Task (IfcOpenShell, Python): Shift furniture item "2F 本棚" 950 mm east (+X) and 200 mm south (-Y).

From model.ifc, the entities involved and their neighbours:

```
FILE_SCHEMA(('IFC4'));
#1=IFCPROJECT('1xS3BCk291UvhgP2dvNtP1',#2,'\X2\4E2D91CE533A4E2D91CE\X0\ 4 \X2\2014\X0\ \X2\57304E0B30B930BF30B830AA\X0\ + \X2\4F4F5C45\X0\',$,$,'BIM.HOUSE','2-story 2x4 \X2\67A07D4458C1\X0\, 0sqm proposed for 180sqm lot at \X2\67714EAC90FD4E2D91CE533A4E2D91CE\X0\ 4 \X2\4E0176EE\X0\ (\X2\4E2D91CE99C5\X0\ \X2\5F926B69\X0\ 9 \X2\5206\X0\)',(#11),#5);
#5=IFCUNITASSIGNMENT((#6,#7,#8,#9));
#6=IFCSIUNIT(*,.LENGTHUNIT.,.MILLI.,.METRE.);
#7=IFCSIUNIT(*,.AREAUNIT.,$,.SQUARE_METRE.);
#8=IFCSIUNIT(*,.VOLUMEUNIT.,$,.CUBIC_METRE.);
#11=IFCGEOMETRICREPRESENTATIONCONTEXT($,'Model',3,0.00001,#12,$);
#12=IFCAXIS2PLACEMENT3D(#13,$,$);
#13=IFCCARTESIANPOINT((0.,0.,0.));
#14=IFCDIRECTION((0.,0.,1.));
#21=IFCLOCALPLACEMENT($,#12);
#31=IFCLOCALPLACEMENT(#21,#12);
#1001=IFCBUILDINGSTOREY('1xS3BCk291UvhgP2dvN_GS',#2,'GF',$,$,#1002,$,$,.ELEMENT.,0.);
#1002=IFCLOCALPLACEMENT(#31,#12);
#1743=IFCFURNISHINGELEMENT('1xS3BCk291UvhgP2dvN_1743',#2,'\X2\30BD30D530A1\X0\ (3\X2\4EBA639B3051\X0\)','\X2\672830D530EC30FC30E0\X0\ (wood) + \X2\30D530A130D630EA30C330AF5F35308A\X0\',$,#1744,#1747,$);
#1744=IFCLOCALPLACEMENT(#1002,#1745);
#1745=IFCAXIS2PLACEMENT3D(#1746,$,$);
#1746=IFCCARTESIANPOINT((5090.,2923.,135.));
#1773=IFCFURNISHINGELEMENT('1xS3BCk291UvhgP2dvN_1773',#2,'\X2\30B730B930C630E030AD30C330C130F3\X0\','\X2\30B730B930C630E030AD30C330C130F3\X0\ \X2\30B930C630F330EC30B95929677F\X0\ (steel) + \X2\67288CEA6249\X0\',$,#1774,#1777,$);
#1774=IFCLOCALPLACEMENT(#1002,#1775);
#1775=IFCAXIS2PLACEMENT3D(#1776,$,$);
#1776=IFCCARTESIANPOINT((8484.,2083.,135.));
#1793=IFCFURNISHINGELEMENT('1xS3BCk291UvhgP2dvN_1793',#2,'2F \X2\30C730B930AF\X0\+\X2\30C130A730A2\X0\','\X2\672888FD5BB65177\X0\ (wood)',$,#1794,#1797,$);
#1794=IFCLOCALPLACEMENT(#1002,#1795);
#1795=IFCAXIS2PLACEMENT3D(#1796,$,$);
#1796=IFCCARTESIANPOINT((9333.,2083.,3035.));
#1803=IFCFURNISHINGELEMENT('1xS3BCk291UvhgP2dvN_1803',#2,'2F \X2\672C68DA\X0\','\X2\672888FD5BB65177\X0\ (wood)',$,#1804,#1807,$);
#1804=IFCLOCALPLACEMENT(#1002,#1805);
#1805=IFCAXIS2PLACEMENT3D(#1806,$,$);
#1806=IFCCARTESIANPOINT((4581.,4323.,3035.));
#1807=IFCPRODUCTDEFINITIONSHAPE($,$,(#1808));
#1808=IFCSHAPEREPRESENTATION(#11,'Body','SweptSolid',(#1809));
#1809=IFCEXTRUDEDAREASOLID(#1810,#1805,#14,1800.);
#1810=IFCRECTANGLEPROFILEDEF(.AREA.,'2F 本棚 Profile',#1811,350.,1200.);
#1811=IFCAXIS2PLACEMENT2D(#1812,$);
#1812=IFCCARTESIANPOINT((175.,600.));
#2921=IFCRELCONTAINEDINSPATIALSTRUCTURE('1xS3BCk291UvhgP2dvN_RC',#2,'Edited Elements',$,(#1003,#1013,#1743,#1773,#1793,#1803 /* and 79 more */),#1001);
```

```python
import ifcopenshell
import ifcopenshell.api.geometry
import ifcopenshell.util.placement
import ifcopenshell.util.unit

model = ifcopenshell.open("model.ifc")
unit_scale = ifcopenshell.util.unit.calculate_unit_scale(model)

item = model.by_guid("1xS3BCk291UvhgP2dvN_1803")
matrix = ifcopenshell.util.placement.get_local_placement(item.ObjectPlacement)
matrix[0, 3] += 0.95 / unit_scale
matrix[1, 3] -= 0.2 / unit_scale
ifcopenshell.api.geometry.edit_object_placement(model, product=item, matrix=matrix, is_si=False)

print(ifcopenshell.util.placement.get_local_placement(item.ObjectPlacement).round(3) + 0.0)

model.write("model_updated.ifc")
```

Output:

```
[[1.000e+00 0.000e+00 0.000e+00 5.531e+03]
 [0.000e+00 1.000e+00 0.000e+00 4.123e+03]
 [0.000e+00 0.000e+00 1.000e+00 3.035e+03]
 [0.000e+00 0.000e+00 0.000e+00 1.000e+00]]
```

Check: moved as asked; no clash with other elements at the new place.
